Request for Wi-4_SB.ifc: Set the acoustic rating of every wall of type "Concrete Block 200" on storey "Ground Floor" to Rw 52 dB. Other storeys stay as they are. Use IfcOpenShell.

First a look at what the model holds.

```python
import ifcopenshell
import ifcopenshell.util.element

model = ifcopenshell.open("Wi-4_SB.ifc")
print(model.schema)
storey = next(s for s in model.by_type("IfcBuildingStorey") if s.Name == "Ground Floor")
walls = [e for e in ifcopenshell.util.element.get_decomposition(storey) if e.is_a("IfcWall")]
seen = {}
for e in walls:
    element_type = ifcopenshell.util.element.get_type(e)
    key = (element_type.Name if element_type != e and element_type else None, ifcopenshell.util.element.get_pset(e, "Pset_WallCommon", "AcousticRating"))
    seen[key] = seen.get(key, 0) + 1
for (name, value), count in sorted(seen.items(), key=str):
    print(count, "x", name, "|", value)
```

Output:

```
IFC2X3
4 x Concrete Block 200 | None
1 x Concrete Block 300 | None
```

```python
import ifcopenshell
import ifcopenshell.api.pset
import ifcopenshell.util.element

model = ifcopenshell.open("Wi-4_SB.ifc")

storey = next(s for s in model.by_type("IfcBuildingStorey") if s.Name == "Ground Floor")
walls = [e for e in ifcopenshell.util.element.get_decomposition(storey) if e.is_a("IfcWall")]

count = 0
for e in walls:
    element_type = ifcopenshell.util.element.get_type(e)
    if element_type in (None, e) or element_type.Name != "Concrete Block 200":
        continue
    # add_pset returns the element's existing set when there is one.
    pset = ifcopenshell.api.pset.add_pset(model, product=e, name="Pset_WallCommon")
    ifcopenshell.api.pset.edit_pset(model, pset=pset, properties={"AcousticRating": "Rw 52 dB"})
    count += 1

print(count, "walls updated")

model.write("Wi-4_SB_edited.ifc")
```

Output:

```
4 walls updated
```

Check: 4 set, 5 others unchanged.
